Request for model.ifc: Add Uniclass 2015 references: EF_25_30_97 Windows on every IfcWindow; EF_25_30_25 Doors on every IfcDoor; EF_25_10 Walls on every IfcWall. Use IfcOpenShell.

First a look at what the model holds.

```python
import ifcopenshell

model = ifcopenshell.open("model.ifc")
print(model.schema)
print("classifications:", [c.Name for c in model.by_type("IfcClassification")])
for ifc_class in ("IfcDoor", "IfcRoof", "IfcStair", "IfcWall", "IfcWindow"):
    print(ifc_class, len(model.by_type(ifc_class)))
```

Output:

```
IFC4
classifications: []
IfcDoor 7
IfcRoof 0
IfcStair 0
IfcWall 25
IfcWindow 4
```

```python
import ifcopenshell
import ifcopenshell.api.classification

model = ifcopenshell.open("model.ifc")

system = ifcopenshell.api.classification.add_classification(model, classification="Uniclass 2015")

codes = {
    "IfcWindow": ("EF_25_30_97", "Windows"),
    "IfcDoor": ("EF_25_30_25", "Doors"),
    "IfcWall": ("EF_25_10", "Walls"),
}
for ifc_class, (code, name) in codes.items():
    products = model.by_type(ifc_class)
    ifcopenshell.api.classification.add_reference(
        model, products=products, classification=system, identification=code, name=name
    )
    print(code, len(products))

model.write("model_updated.ifc")
```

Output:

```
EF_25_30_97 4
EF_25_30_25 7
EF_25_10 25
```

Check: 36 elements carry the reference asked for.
